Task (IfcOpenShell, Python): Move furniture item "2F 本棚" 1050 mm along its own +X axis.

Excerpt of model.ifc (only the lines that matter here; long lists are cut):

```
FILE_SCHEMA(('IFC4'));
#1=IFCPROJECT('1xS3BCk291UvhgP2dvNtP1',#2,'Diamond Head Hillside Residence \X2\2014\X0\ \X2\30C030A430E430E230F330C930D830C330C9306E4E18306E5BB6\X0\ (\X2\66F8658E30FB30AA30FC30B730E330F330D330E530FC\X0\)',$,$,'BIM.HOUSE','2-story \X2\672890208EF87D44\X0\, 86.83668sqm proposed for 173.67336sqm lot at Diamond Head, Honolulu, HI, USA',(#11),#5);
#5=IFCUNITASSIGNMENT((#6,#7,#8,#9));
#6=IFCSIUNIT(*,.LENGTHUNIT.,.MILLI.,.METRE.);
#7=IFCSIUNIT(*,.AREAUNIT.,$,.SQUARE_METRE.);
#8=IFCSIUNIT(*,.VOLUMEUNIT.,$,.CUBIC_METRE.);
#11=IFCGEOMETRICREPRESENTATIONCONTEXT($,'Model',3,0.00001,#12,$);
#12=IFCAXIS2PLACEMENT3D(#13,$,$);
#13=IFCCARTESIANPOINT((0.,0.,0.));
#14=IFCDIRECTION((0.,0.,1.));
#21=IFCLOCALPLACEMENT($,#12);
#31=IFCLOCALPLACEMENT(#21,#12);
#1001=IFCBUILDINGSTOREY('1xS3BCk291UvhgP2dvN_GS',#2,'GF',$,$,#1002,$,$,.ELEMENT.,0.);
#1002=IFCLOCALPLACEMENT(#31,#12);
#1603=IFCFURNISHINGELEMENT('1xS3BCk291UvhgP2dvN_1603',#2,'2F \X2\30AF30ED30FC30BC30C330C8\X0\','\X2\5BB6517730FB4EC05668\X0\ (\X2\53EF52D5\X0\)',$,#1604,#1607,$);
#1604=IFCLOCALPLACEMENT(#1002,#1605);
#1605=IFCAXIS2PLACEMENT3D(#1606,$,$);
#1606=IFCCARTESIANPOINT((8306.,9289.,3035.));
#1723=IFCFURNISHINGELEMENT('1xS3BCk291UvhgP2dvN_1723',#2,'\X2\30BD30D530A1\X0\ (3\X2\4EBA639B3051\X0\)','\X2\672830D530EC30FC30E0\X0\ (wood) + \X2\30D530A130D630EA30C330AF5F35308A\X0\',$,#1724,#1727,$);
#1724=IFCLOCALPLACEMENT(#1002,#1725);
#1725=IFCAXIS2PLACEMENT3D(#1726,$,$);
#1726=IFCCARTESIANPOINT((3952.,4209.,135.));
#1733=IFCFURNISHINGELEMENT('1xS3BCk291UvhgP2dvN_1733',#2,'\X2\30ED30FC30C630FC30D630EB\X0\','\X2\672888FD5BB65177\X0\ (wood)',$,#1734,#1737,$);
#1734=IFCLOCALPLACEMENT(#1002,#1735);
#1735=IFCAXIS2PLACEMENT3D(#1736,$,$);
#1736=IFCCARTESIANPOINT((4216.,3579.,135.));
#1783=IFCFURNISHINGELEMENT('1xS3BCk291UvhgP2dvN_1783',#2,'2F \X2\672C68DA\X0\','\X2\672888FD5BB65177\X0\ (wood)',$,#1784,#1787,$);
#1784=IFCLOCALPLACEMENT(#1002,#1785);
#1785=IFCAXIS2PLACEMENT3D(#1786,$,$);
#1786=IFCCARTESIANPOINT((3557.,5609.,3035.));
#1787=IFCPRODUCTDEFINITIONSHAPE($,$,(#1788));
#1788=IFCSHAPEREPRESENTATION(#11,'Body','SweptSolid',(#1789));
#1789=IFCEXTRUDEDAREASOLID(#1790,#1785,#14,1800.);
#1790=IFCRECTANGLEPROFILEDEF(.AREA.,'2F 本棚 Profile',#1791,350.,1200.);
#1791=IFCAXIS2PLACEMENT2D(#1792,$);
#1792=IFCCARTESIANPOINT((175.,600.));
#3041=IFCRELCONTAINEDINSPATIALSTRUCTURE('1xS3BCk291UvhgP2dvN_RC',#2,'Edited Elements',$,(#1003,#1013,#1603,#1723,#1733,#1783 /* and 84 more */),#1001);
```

```python
import ifcopenshell
import ifcopenshell.api.geometry
import ifcopenshell.util.placement
import ifcopenshell.util.unit

model = ifcopenshell.open("model.ifc")
unit_scale = ifcopenshell.util.unit.calculate_unit_scale(model)

item = model.by_id(1783)
matrix = ifcopenshell.util.placement.get_local_placement(item.ObjectPlacement)
matrix[:3, 3] += matrix[:3, 0] * 1.05 / unit_scale
ifcopenshell.api.geometry.edit_object_placement(model, product=item, matrix=matrix, is_si=False)

print(ifcopenshell.util.placement.get_local_placement(item.ObjectPlacement).round(3) + 0.0)

model.write("model_rev.ifc")
```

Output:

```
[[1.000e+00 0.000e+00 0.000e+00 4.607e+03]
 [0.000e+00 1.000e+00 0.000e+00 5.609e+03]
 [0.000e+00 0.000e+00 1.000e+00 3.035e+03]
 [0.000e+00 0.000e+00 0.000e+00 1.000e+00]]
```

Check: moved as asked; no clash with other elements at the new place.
